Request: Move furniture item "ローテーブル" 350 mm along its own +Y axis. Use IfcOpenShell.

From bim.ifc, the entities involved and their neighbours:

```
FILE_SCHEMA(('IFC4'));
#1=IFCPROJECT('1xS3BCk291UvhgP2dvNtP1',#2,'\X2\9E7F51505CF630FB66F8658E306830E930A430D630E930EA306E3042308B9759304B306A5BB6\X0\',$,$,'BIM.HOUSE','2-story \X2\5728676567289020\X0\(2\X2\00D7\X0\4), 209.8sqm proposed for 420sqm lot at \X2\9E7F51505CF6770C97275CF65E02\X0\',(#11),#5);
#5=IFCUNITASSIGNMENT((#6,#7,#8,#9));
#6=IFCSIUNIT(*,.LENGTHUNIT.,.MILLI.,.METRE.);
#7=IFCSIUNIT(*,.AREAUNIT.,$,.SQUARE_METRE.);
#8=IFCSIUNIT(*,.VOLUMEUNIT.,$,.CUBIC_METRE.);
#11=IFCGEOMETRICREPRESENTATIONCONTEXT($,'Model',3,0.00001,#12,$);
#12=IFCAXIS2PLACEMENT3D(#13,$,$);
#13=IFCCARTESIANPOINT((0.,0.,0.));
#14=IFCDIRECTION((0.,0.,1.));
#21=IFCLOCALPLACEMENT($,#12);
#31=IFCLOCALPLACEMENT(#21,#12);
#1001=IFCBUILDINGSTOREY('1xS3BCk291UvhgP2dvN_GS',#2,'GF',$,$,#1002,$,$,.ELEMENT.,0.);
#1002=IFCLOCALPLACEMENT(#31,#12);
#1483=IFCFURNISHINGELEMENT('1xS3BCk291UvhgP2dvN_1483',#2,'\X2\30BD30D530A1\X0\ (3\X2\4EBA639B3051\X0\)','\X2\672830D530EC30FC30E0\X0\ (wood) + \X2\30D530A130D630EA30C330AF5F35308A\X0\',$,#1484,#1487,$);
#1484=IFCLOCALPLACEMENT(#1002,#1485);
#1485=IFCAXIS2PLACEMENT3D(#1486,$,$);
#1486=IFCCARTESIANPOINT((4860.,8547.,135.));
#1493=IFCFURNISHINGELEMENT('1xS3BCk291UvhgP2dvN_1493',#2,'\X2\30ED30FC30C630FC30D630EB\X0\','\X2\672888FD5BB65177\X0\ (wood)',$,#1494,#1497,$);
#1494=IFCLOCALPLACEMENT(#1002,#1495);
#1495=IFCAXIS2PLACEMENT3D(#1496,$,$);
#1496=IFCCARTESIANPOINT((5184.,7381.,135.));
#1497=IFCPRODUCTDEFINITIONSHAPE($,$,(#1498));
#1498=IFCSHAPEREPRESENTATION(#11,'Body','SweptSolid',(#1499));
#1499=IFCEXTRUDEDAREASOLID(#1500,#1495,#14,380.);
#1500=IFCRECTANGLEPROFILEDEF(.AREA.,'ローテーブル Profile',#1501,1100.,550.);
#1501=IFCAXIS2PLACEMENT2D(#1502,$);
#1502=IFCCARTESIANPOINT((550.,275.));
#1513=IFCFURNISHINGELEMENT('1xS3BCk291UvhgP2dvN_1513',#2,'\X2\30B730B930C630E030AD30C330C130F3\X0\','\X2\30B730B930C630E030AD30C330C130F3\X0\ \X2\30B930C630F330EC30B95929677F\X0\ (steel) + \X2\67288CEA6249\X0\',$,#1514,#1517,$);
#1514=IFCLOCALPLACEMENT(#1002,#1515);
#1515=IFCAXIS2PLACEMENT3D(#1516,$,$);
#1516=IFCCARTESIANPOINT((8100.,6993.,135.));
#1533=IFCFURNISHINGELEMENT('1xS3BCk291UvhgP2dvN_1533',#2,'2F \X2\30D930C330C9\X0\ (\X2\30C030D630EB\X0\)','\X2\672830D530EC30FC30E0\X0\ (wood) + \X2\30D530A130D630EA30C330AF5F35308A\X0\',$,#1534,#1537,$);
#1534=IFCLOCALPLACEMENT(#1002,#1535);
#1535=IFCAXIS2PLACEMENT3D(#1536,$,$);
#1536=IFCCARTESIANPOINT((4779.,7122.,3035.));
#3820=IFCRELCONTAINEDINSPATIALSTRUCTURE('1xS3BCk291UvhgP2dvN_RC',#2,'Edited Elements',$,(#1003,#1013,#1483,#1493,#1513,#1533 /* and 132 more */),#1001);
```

```python
import ifcopenshell
import ifcopenshell.api.geometry
import ifcopenshell.util.placement
import ifcopenshell.util.unit

model = ifcopenshell.open("bim.ifc")
unit_scale = ifcopenshell.util.unit.calculate_unit_scale(model)

item = model.by_guid("1xS3BCk291UvhgP2dvN_1493")
matrix = ifcopenshell.util.placement.get_local_placement(item.ObjectPlacement)
matrix[:3, 3] += matrix[:3, 1] * 0.35 / unit_scale
ifcopenshell.api.geometry.edit_object_placement(model, product=item, matrix=matrix, is_si=False)

print(ifcopenshell.util.placement.get_local_placement(item.ObjectPlacement).round(3) + 0.0)

model.write("bim_edited.ifc")
```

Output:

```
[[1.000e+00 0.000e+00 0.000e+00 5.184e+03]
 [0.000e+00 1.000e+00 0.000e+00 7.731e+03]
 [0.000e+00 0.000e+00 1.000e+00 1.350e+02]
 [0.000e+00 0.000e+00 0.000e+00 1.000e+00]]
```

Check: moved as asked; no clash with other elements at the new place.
